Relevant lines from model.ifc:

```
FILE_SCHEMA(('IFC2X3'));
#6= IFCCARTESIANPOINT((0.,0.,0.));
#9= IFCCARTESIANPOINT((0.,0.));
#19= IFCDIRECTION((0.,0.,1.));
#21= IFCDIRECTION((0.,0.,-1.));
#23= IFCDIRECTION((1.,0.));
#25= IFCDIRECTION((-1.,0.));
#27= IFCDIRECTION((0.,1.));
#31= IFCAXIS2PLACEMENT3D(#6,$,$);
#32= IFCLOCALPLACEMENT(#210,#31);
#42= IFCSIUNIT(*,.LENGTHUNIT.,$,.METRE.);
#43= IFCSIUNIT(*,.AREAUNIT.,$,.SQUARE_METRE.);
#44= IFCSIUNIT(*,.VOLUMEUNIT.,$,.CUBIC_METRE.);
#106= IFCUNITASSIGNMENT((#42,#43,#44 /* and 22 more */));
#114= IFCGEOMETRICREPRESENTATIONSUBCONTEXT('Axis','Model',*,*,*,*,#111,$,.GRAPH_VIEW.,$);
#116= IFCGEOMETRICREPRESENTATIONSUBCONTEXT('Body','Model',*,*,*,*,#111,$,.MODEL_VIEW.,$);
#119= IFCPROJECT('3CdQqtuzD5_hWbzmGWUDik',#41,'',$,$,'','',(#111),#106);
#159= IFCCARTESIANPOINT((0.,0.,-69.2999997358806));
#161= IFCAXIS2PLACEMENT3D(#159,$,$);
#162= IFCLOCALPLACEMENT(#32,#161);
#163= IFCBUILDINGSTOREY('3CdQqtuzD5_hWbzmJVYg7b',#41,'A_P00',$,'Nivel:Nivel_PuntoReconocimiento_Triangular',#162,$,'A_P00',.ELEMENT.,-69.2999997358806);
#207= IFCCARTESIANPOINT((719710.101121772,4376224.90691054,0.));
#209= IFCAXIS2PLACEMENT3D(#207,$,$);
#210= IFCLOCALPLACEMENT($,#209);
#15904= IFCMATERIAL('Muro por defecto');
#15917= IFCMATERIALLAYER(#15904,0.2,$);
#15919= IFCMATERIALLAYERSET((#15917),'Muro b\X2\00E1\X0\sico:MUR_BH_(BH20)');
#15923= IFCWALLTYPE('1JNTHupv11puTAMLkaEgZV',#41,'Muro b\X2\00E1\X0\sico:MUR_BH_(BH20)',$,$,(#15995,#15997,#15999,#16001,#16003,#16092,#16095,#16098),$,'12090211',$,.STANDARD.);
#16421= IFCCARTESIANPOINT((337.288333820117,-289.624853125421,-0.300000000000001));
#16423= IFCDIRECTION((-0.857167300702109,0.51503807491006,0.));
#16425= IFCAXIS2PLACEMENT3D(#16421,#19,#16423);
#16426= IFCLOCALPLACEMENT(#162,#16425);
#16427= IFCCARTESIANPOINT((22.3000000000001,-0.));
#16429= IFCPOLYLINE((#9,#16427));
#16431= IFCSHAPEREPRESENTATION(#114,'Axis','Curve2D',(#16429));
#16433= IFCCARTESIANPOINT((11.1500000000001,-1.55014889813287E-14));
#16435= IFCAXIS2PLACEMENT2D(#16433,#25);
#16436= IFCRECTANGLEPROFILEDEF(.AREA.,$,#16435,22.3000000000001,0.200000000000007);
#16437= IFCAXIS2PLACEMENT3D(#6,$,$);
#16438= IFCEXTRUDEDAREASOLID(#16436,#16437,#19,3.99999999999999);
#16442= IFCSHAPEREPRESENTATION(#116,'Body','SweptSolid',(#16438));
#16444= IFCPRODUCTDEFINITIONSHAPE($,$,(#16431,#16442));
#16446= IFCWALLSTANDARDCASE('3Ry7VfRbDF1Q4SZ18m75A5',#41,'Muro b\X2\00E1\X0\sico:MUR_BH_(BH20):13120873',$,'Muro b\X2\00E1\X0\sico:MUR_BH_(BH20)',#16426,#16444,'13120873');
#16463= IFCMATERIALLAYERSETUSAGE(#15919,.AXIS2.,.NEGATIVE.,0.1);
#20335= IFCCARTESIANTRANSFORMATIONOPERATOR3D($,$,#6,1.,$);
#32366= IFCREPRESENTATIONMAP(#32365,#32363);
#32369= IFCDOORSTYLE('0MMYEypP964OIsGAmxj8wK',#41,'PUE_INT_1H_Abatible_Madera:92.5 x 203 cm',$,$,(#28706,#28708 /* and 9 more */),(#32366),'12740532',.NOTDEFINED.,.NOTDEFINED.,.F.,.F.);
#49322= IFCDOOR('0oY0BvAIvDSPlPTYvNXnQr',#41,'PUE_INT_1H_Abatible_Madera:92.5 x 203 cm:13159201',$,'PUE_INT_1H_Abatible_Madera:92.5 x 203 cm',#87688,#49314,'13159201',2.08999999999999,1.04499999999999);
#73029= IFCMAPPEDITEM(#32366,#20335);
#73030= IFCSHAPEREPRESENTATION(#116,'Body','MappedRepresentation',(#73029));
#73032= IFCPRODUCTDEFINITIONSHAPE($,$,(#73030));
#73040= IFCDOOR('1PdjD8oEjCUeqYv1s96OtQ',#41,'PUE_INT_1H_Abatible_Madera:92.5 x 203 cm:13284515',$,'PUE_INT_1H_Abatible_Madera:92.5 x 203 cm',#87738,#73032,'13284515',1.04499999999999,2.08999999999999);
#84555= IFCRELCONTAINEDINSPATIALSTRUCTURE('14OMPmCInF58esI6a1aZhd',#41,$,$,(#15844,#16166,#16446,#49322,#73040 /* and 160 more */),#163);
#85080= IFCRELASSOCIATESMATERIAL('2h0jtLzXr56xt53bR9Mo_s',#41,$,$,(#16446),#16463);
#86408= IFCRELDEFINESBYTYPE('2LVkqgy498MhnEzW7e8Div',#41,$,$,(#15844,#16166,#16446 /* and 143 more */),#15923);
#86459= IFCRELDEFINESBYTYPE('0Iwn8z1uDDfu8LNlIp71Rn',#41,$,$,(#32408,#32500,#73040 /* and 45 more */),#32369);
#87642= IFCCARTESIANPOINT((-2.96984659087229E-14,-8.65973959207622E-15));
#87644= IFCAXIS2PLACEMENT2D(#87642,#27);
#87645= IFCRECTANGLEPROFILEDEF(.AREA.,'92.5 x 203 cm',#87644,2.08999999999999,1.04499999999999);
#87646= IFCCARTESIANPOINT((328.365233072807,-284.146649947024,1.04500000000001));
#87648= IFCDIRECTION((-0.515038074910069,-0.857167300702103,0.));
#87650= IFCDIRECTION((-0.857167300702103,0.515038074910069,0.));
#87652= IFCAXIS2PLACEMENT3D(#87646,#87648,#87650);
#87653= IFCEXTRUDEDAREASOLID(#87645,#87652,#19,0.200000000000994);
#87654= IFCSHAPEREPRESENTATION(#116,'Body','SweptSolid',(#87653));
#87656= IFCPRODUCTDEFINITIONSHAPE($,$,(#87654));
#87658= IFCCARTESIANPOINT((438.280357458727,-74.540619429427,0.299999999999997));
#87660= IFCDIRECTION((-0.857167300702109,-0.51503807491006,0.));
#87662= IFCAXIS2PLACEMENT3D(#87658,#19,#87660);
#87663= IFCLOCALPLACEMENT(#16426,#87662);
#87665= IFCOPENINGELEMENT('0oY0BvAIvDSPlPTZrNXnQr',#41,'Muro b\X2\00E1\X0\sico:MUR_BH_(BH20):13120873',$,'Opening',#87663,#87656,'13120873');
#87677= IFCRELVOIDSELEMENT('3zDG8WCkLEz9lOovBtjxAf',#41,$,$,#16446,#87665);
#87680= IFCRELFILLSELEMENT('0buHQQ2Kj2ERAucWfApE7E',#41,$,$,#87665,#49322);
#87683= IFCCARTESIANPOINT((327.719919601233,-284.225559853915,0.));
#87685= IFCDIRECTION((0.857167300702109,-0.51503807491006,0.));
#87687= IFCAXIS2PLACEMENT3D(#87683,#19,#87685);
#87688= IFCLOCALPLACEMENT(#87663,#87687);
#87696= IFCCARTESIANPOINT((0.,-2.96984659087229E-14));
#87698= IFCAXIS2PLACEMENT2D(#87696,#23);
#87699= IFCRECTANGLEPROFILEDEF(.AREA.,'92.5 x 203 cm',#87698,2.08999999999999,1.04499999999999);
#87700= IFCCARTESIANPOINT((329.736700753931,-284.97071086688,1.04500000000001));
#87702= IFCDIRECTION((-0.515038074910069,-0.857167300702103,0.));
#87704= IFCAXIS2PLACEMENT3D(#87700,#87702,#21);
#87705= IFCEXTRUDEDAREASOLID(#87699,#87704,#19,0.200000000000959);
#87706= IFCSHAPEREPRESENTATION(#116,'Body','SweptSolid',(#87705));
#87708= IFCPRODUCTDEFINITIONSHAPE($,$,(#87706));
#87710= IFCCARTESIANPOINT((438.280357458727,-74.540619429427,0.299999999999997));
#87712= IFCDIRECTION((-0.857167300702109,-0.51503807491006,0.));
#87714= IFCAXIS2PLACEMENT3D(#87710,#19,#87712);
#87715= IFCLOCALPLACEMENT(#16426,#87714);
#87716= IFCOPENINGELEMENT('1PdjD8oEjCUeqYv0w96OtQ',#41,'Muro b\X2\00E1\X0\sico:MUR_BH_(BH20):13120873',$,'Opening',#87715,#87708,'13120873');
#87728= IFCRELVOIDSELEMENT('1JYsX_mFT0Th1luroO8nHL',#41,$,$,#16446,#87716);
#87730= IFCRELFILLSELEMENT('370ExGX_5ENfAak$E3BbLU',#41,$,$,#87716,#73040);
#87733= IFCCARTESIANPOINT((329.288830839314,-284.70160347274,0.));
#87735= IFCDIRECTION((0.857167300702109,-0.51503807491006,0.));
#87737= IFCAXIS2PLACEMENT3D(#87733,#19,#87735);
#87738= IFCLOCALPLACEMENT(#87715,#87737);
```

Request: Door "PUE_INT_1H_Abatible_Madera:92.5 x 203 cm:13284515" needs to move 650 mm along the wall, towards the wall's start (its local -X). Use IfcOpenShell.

```python
import ifcopenshell
import ifcopenshell.api.geometry
import ifcopenshell.util.placement
import ifcopenshell.util.unit

model = ifcopenshell.open("model.ifc")
unit_scale = ifcopenshell.util.unit.calculate_unit_scale(model)

door = model.by_id(73040)
opening = door.FillsVoids[0].RelatingOpeningElement
wall = opening.VoidsElements[0].RelatingBuildingElement

wall_matrix = ifcopenshell.util.placement.get_local_placement(wall.ObjectPlacement)
shift = wall_matrix[:3, 0] * -0.65 / unit_scale
before = ifcopenshell.util.placement.get_local_placement(door.ObjectPlacement)[:3, 3].copy()

# The door is placed relative to its opening, so it follows when the opening moves.
matrix = ifcopenshell.util.placement.get_local_placement(opening.ObjectPlacement)
matrix[:3, 3] += shift
ifcopenshell.api.geometry.edit_object_placement(
    model, product=opening, matrix=matrix, is_si=False, should_transform_children=True
)

after = ifcopenshell.util.placement.get_local_placement(door.ObjectPlacement)[:3, 3]
print("door moved by", (after - before).round(3) + 0.0)

model.write("model_rev.ifc")
```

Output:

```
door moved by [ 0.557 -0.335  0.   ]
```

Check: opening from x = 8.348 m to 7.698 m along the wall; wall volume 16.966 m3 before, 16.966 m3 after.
